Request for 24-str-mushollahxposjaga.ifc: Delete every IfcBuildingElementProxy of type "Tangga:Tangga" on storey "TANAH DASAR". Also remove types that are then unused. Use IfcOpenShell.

First a look at what the model holds.

```python
import ifcopenshell
import ifcopenshell.util.element

model = ifcopenshell.open("24-str-mushollahxposjaga.ifc")
print(model.schema)
storey = next(s for s in model.by_type("IfcBuildingStorey") if s.Name == "TANAH DASAR")
proxies = [e for e in ifcopenshell.util.element.get_decomposition(storey) if e.is_a("IfcBuildingElementProxy")]
seen = {}
for e in proxies:
    element_type = ifcopenshell.util.element.get_type(e)
    name = element_type.Name if element_type not in (None, e) else None
    seen[name] = seen.get(name, 0) + 1
for name, count in sorted(seen.items(), key=str):
    print(count, "x", name)
```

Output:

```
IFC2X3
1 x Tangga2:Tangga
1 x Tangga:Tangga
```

```python
import ifcopenshell
import ifcopenshell.api.root
import ifcopenshell.util.element

model = ifcopenshell.open("24-str-mushollahxposjaga.ifc")

storey = next(s for s in model.by_type("IfcBuildingStorey") if s.Name == "TANAH DASAR")
proxies = [e for e in ifcopenshell.util.element.get_decomposition(storey) if e.is_a("IfcBuildingElementProxy")]
targets = [e for e in proxies if (t := ifcopenshell.util.element.get_type(e)) not in (None, e) and t.Name == "Tangga:Tangga"]
types = {ifcopenshell.util.element.get_type(e) for e in targets} - {None, *targets}

for e in targets:
    ifcopenshell.api.root.remove_product(model, product=e)
print(len(targets), "removed")

unused = [t for t in types if not ifcopenshell.util.element.get_types(t)]
for t in unused:
    ifcopenshell.api.root.remove_product(model, product=t)
print(len(unused), "unused types removed")

model.write("24-str-mushollahxposjaga_edited.ifc")
```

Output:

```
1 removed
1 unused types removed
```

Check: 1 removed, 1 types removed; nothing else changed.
